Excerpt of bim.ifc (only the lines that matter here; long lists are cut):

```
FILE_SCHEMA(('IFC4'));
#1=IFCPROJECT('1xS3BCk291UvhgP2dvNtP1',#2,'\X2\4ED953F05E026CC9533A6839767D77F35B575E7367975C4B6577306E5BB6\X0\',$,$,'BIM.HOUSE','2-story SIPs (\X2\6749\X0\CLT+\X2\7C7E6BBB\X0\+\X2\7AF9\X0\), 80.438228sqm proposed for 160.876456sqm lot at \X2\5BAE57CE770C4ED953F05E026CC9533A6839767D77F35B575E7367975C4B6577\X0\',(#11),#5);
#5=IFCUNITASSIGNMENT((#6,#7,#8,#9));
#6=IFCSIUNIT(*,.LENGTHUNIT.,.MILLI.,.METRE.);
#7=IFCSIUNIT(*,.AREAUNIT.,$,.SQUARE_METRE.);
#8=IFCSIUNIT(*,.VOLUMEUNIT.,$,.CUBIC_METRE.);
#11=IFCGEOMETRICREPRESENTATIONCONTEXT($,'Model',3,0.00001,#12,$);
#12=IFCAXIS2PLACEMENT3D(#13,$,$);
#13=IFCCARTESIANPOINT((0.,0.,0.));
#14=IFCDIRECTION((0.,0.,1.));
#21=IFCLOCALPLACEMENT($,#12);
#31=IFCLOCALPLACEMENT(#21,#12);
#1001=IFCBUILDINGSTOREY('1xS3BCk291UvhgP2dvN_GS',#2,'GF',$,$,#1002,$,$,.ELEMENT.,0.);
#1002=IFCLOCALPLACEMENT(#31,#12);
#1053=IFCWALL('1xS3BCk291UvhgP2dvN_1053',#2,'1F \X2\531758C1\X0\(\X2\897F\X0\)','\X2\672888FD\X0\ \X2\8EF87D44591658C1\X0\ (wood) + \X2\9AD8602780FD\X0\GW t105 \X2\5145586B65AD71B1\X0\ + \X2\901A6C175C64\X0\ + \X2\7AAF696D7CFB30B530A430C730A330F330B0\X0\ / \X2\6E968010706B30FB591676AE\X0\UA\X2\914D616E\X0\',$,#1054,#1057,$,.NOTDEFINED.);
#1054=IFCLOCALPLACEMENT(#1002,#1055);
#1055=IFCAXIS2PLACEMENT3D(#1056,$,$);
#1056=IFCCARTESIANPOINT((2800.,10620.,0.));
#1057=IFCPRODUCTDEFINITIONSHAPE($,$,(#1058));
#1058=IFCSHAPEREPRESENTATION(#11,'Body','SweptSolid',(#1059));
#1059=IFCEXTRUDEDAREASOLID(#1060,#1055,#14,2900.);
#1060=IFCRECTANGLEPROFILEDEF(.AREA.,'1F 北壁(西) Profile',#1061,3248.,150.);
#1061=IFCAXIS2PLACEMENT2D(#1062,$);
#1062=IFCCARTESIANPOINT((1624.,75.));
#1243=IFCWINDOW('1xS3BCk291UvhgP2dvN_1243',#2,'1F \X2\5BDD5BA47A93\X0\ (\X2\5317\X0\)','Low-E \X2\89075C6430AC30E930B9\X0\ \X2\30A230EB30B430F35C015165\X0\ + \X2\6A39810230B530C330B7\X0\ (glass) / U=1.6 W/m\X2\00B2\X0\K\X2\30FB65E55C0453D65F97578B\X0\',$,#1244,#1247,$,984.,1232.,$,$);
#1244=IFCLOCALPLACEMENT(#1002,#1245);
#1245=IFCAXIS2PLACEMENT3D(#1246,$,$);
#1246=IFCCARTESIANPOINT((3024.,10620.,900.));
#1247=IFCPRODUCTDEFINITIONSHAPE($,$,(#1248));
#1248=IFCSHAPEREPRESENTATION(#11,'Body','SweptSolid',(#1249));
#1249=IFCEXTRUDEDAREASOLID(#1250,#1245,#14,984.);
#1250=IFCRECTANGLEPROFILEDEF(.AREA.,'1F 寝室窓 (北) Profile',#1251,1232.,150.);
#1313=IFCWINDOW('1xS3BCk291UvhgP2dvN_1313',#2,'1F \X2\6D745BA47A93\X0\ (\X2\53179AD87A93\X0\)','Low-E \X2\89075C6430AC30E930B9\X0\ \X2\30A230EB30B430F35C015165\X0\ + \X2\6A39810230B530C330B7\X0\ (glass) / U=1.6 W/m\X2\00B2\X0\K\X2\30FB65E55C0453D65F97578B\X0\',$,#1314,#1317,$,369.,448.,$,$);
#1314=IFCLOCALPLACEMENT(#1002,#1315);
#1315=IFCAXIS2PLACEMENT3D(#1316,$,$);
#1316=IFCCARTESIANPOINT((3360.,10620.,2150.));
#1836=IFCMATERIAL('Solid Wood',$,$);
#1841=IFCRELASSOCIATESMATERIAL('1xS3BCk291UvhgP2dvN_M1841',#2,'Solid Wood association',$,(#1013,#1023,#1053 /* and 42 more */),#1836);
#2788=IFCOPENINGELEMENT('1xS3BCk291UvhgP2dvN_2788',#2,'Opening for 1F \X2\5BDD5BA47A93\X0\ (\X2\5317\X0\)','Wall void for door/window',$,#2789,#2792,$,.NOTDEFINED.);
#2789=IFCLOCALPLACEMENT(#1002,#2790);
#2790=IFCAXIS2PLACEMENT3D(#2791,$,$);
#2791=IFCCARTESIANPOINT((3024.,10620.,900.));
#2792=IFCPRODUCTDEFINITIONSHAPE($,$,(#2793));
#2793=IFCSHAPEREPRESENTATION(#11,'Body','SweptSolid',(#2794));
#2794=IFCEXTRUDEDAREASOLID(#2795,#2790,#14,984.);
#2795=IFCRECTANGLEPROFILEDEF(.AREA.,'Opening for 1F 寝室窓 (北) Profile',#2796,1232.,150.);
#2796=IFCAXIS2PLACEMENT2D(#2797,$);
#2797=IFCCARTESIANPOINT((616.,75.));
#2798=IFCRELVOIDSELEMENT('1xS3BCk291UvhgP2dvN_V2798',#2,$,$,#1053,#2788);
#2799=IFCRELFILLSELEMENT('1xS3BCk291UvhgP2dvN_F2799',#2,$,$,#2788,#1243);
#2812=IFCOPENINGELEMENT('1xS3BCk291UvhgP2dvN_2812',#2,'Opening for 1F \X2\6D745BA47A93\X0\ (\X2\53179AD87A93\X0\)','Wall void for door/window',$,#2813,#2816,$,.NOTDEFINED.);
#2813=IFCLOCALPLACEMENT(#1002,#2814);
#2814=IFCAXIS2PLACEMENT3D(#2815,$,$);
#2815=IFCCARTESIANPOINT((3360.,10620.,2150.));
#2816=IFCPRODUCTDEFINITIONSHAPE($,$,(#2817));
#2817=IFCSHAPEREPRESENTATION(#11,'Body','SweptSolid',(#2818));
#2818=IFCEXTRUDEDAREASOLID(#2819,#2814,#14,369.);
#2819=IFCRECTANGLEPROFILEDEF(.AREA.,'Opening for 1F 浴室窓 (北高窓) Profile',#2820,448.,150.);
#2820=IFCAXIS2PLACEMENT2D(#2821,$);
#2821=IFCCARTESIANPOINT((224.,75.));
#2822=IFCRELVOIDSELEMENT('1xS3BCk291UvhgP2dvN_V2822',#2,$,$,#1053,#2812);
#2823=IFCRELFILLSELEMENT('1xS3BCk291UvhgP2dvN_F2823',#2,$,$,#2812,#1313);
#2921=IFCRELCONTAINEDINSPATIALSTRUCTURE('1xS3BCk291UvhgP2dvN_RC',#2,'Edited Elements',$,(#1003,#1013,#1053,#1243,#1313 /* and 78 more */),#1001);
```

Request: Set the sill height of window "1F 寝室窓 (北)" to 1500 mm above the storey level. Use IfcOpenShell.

```python
import numpy as np
import ifcopenshell
import ifcopenshell.api.geometry
import ifcopenshell.geom
import ifcopenshell.util.element
import ifcopenshell.util.placement
import ifcopenshell.util.shape
import ifcopenshell.util.unit

model = ifcopenshell.open("bim.ifc")
unit_scale = ifcopenshell.util.unit.calculate_unit_scale(model)

window = model.by_guid("1xS3BCk291UvhgP2dvN_1243")
opening = window.FillsVoids[0].RelatingOpeningElement
storey = ifcopenshell.util.element.get_container(window, ifc_class="IfcBuildingStorey")
level = ifcopenshell.util.placement.get_local_placement(storey.ObjectPlacement)[2, 3]

# The opening's origin need not be at the sill, so measure its lowest point.
shape = ifcopenshell.geom.create_shape(ifcopenshell.geom.settings(), opening)
bottom = ifcopenshell.util.shape.get_shape_bottom_elevation(shape, shape.geometry) / unit_scale
dz = level + 1.5 / unit_scale - bottom

shift = np.array([0.0, 0.0, dz])
# The window is not placed relative to its opening, so move both.
for product in (opening, window):
    matrix = ifcopenshell.util.placement.get_local_placement(product.ObjectPlacement)
    matrix[:3, 3] += shift
    ifcopenshell.api.geometry.edit_object_placement(model, product=product, matrix=matrix, is_si=False)

print(f"moved by {dz * unit_scale:+.3f} m")

model.write("bim_updated.ifc")
```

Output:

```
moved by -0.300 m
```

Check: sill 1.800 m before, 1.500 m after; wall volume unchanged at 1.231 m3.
